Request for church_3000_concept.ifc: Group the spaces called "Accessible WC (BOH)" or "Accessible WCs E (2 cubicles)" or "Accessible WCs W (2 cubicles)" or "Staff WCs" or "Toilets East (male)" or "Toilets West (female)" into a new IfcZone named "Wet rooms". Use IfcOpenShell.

First a look at what the model holds.

```python
import ifcopenshell

model = ifcopenshell.open("church_3000_concept.ifc")
print(model.schema)
seen = {}
for space in model.by_type("IfcSpace"):
    seen[space.LongName] = seen.get(space.LongName, 0) + 1
for name, count in sorted(seen.items(), key=str):
    print(count, "x", name)
print("zones:", [z.Name for z in model.by_type("IfcZone")][:20])
```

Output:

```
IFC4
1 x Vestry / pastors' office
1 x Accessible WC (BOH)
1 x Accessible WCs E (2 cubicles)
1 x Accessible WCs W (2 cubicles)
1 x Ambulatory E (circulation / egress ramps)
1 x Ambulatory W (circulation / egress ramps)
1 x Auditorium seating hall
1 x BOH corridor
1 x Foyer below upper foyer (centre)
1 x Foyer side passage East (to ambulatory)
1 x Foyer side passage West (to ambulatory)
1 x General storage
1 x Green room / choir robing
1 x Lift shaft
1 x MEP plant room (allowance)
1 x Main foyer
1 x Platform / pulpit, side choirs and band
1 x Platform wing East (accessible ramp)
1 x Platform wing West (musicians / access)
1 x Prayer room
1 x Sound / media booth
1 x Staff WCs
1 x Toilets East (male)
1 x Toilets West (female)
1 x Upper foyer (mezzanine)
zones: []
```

```python
import ifcopenshell
import ifcopenshell.api.group
import ifcopenshell.api.root

model = ifcopenshell.open("church_3000_concept.ifc")

names = {"Accessible WC (BOH)", "Accessible WCs E (2 cubicles)", "Accessible WCs W (2 cubicles)", "Staff WCs", "Toilets East (male)", "Toilets West (female)"}
spaces = [s for s in model.by_type("IfcSpace") if s.LongName in names]

zone = ifcopenshell.api.root.create_entity(model, ifc_class="IfcZone", name="Wet rooms")
ifcopenshell.api.group.assign_group(model, products=spaces, group=zone)
print(len(spaces), "spaces in", zone.Name)

model.write("church_3000_concept_updated.ifc")
```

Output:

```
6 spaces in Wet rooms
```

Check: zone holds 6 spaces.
